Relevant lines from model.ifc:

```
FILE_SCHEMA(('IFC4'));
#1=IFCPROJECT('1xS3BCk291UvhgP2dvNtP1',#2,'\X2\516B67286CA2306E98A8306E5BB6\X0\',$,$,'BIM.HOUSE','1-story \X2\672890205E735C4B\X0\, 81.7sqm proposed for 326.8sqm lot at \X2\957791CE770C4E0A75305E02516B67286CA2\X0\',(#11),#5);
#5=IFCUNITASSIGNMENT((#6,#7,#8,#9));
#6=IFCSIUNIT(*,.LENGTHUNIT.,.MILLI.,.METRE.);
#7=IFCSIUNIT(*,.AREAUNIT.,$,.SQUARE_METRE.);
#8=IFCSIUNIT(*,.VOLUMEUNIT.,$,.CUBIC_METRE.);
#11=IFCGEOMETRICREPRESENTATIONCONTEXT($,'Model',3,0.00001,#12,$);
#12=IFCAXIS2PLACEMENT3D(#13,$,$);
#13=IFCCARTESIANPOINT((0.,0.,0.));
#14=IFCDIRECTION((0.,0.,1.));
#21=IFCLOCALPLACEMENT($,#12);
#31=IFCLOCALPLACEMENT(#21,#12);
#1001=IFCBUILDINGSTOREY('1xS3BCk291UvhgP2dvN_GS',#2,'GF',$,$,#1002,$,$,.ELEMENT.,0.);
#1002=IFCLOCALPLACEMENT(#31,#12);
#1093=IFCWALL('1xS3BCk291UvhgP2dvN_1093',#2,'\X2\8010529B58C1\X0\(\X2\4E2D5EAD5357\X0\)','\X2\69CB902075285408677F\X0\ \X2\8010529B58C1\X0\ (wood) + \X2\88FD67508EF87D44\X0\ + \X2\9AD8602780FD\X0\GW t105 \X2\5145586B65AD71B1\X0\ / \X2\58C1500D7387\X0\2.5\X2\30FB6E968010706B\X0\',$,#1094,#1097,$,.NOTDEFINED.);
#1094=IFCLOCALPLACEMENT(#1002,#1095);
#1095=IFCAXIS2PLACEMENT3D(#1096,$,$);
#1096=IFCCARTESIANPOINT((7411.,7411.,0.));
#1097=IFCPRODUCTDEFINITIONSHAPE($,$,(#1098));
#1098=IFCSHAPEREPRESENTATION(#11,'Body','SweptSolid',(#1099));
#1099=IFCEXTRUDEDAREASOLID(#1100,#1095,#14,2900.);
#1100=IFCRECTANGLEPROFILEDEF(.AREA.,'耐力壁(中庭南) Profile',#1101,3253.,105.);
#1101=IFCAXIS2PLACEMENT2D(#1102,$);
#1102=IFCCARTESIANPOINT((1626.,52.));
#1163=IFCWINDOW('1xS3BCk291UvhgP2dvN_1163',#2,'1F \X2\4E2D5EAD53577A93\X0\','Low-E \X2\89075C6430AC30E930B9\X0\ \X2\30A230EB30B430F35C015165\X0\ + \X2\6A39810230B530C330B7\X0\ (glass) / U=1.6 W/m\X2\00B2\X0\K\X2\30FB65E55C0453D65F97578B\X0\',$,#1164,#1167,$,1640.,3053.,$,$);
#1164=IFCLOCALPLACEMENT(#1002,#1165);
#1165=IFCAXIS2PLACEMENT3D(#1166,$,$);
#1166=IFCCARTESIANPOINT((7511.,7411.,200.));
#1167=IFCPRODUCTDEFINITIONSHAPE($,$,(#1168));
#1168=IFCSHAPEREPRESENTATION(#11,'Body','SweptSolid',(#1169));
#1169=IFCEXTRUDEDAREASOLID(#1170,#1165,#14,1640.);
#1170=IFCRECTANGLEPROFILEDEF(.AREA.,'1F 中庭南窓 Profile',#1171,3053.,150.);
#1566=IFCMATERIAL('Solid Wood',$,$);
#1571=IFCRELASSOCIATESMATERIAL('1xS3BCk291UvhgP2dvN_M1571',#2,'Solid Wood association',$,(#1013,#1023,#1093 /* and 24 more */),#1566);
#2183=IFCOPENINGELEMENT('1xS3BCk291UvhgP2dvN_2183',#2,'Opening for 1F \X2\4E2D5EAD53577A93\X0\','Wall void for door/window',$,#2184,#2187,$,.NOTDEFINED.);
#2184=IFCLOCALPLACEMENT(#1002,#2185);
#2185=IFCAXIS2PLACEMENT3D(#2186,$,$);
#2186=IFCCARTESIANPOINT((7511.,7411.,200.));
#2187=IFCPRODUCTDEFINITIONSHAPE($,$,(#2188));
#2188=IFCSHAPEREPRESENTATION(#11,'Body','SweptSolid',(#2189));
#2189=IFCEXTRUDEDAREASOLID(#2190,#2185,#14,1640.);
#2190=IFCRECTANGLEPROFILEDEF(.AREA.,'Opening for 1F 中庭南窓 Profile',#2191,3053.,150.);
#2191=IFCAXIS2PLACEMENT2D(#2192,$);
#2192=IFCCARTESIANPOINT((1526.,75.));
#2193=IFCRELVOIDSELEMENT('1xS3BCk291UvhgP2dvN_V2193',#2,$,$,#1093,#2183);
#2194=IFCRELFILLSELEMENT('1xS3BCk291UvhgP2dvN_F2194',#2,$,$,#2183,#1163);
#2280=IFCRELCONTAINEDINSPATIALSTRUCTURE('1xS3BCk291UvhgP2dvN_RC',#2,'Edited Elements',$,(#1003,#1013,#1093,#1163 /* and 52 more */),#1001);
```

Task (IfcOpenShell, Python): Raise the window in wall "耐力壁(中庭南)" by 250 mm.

```python
import numpy as np
import ifcopenshell
import ifcopenshell.api.geometry
import ifcopenshell.util.placement
import ifcopenshell.util.unit

model = ifcopenshell.open("model.ifc")
unit_scale = ifcopenshell.util.unit.calculate_unit_scale(model)

window = model.by_guid("1xS3BCk291UvhgP2dvN_1163")
opening = window.FillsVoids[0].RelatingOpeningElement
dz = 0.25 / unit_scale

shift = np.array([0.0, 0.0, dz])
# The window is not placed relative to its opening, so move both.
for product in (opening, window):
    matrix = ifcopenshell.util.placement.get_local_placement(product.ObjectPlacement)
    matrix[:3, 3] += shift
    ifcopenshell.api.geometry.edit_object_placement(model, product=product, matrix=matrix, is_si=False)

print(f"moved by {dz * unit_scale:+.3f} m")

model.write("model_rev.ifc")
```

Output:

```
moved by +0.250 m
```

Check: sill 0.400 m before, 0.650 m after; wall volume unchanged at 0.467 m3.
